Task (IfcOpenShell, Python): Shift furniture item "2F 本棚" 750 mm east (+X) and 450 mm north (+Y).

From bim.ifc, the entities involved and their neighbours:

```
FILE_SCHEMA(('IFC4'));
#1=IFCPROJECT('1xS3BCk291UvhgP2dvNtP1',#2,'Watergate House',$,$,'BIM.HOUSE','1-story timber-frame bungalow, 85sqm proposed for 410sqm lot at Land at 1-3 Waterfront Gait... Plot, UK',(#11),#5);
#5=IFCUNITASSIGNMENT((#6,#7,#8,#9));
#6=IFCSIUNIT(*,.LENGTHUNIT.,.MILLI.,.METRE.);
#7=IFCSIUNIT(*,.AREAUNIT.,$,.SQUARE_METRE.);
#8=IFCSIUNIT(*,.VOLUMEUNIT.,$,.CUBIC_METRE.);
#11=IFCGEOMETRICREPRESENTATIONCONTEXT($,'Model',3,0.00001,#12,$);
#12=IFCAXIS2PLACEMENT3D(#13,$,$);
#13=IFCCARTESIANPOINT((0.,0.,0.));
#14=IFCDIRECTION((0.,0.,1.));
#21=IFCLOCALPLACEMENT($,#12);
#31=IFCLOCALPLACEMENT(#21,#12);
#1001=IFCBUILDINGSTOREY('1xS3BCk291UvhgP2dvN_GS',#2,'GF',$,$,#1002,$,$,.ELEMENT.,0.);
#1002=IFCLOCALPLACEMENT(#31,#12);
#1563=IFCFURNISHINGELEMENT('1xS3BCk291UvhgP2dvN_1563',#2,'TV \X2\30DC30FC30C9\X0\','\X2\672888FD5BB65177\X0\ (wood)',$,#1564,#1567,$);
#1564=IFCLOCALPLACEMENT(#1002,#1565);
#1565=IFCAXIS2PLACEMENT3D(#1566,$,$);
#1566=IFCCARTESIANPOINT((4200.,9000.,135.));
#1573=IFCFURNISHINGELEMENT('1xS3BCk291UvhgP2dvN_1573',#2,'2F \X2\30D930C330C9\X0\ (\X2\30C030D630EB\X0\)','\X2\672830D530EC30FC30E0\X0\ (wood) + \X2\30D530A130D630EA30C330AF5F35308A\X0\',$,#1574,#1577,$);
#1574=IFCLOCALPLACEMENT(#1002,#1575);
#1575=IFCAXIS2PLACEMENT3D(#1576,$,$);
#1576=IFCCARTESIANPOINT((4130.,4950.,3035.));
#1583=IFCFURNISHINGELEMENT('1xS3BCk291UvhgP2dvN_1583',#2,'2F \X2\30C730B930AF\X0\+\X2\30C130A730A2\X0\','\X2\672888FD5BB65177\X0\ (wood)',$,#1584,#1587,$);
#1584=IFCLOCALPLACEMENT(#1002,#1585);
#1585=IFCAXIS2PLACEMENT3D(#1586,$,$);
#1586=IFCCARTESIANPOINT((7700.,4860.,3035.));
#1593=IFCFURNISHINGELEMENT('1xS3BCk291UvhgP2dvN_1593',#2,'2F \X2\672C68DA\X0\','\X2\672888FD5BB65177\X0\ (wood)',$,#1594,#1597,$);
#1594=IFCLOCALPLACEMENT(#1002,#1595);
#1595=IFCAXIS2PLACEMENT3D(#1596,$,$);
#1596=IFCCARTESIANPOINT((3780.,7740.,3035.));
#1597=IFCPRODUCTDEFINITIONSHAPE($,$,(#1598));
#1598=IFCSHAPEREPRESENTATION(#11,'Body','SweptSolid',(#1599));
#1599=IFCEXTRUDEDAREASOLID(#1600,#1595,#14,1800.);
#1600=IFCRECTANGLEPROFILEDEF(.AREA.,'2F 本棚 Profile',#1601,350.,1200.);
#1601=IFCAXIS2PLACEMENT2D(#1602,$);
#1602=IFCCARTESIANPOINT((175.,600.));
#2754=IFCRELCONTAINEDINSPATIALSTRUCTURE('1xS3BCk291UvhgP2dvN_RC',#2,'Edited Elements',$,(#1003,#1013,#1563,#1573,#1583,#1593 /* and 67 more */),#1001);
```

```python
import ifcopenshell
import ifcopenshell.api.geometry
import ifcopenshell.util.placement
import ifcopenshell.util.unit

model = ifcopenshell.open("bim.ifc")
unit_scale = ifcopenshell.util.unit.calculate_unit_scale(model)

item = model.by_guid("1xS3BCk291UvhgP2dvN_1593")
matrix = ifcopenshell.util.placement.get_local_placement(item.ObjectPlacement)
matrix[0, 3] += 0.75 / unit_scale
matrix[1, 3] += 0.45 / unit_scale
ifcopenshell.api.geometry.edit_object_placement(model, product=item, matrix=matrix, is_si=False)

print(ifcopenshell.util.placement.get_local_placement(item.ObjectPlacement).round(3) + 0.0)

model.write("bim-out.ifc")
```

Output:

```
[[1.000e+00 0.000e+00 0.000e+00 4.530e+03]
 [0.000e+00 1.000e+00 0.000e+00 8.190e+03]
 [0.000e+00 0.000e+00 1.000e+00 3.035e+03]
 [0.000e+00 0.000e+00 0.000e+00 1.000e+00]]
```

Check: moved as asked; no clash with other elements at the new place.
